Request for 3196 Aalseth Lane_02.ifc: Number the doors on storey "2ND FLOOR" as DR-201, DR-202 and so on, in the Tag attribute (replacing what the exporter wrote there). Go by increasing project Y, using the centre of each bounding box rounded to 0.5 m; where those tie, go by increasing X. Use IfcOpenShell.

First a look at what the model holds.

```python
import ifcopenshell
import ifcopenshell.util.element
import ifcopenshell.util.placement

model = ifcopenshell.open("3196 Aalseth Lane_02.ifc")
print(model.schema)
storey = next(s for s in model.by_type("IfcBuildingStorey") if s.Name == "2ND FLOOR")
doors = [e for e in ifcopenshell.util.element.get_decomposition(storey) if e.is_a("IfcDoor")]
for e in sorted(doors, key=lambda e: e.id()):
    origin = ifcopenshell.util.placement.get_local_placement(e.ObjectPlacement)[:3, 3]
    print(e.id(), e.Tag, e.Name, origin.round(2) + 0.0, sep=" | ")
```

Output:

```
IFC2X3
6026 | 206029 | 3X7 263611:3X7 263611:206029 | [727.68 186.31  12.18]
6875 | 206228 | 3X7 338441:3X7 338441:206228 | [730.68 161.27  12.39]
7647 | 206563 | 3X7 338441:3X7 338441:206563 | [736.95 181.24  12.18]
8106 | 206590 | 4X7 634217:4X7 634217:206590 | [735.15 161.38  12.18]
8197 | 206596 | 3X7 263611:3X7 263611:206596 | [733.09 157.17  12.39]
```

```python
import ifcopenshell
import ifcopenshell.geom
import ifcopenshell.util.element
import ifcopenshell.util.shape

model = ifcopenshell.open("3196 Aalseth Lane_02.ifc")
settings = ifcopenshell.geom.settings()
settings.set("use-world-coords", True)


def centre(element):
    shape = ifcopenshell.geom.create_shape(settings, element)
    return ifcopenshell.util.shape.get_bbox_centroid(shape.geometry)


storey = next(s for s in model.by_type("IfcBuildingStorey") if s.Name == "2ND FLOOR")
doors = [e for e in ifcopenshell.util.element.get_decomposition(storey) if e.is_a("IfcDoor")]

# Insertion points can sit at a corner or the storey origin, so sort by the geometry (in metres).
centres = {e: centre(e) for e in doors}
doors.sort(key=lambda e: (round(centres[e][1] / 0.5), centres[e][0]))

for i, e in enumerate(doors, start=1):
    number = f"DR-2{i:02d}"
    e.Tag = number
    print(e.id(), number)

model.write("3196 Aalseth Lane_02_rev.ifc")
```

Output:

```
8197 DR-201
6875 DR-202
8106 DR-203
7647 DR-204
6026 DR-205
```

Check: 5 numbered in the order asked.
